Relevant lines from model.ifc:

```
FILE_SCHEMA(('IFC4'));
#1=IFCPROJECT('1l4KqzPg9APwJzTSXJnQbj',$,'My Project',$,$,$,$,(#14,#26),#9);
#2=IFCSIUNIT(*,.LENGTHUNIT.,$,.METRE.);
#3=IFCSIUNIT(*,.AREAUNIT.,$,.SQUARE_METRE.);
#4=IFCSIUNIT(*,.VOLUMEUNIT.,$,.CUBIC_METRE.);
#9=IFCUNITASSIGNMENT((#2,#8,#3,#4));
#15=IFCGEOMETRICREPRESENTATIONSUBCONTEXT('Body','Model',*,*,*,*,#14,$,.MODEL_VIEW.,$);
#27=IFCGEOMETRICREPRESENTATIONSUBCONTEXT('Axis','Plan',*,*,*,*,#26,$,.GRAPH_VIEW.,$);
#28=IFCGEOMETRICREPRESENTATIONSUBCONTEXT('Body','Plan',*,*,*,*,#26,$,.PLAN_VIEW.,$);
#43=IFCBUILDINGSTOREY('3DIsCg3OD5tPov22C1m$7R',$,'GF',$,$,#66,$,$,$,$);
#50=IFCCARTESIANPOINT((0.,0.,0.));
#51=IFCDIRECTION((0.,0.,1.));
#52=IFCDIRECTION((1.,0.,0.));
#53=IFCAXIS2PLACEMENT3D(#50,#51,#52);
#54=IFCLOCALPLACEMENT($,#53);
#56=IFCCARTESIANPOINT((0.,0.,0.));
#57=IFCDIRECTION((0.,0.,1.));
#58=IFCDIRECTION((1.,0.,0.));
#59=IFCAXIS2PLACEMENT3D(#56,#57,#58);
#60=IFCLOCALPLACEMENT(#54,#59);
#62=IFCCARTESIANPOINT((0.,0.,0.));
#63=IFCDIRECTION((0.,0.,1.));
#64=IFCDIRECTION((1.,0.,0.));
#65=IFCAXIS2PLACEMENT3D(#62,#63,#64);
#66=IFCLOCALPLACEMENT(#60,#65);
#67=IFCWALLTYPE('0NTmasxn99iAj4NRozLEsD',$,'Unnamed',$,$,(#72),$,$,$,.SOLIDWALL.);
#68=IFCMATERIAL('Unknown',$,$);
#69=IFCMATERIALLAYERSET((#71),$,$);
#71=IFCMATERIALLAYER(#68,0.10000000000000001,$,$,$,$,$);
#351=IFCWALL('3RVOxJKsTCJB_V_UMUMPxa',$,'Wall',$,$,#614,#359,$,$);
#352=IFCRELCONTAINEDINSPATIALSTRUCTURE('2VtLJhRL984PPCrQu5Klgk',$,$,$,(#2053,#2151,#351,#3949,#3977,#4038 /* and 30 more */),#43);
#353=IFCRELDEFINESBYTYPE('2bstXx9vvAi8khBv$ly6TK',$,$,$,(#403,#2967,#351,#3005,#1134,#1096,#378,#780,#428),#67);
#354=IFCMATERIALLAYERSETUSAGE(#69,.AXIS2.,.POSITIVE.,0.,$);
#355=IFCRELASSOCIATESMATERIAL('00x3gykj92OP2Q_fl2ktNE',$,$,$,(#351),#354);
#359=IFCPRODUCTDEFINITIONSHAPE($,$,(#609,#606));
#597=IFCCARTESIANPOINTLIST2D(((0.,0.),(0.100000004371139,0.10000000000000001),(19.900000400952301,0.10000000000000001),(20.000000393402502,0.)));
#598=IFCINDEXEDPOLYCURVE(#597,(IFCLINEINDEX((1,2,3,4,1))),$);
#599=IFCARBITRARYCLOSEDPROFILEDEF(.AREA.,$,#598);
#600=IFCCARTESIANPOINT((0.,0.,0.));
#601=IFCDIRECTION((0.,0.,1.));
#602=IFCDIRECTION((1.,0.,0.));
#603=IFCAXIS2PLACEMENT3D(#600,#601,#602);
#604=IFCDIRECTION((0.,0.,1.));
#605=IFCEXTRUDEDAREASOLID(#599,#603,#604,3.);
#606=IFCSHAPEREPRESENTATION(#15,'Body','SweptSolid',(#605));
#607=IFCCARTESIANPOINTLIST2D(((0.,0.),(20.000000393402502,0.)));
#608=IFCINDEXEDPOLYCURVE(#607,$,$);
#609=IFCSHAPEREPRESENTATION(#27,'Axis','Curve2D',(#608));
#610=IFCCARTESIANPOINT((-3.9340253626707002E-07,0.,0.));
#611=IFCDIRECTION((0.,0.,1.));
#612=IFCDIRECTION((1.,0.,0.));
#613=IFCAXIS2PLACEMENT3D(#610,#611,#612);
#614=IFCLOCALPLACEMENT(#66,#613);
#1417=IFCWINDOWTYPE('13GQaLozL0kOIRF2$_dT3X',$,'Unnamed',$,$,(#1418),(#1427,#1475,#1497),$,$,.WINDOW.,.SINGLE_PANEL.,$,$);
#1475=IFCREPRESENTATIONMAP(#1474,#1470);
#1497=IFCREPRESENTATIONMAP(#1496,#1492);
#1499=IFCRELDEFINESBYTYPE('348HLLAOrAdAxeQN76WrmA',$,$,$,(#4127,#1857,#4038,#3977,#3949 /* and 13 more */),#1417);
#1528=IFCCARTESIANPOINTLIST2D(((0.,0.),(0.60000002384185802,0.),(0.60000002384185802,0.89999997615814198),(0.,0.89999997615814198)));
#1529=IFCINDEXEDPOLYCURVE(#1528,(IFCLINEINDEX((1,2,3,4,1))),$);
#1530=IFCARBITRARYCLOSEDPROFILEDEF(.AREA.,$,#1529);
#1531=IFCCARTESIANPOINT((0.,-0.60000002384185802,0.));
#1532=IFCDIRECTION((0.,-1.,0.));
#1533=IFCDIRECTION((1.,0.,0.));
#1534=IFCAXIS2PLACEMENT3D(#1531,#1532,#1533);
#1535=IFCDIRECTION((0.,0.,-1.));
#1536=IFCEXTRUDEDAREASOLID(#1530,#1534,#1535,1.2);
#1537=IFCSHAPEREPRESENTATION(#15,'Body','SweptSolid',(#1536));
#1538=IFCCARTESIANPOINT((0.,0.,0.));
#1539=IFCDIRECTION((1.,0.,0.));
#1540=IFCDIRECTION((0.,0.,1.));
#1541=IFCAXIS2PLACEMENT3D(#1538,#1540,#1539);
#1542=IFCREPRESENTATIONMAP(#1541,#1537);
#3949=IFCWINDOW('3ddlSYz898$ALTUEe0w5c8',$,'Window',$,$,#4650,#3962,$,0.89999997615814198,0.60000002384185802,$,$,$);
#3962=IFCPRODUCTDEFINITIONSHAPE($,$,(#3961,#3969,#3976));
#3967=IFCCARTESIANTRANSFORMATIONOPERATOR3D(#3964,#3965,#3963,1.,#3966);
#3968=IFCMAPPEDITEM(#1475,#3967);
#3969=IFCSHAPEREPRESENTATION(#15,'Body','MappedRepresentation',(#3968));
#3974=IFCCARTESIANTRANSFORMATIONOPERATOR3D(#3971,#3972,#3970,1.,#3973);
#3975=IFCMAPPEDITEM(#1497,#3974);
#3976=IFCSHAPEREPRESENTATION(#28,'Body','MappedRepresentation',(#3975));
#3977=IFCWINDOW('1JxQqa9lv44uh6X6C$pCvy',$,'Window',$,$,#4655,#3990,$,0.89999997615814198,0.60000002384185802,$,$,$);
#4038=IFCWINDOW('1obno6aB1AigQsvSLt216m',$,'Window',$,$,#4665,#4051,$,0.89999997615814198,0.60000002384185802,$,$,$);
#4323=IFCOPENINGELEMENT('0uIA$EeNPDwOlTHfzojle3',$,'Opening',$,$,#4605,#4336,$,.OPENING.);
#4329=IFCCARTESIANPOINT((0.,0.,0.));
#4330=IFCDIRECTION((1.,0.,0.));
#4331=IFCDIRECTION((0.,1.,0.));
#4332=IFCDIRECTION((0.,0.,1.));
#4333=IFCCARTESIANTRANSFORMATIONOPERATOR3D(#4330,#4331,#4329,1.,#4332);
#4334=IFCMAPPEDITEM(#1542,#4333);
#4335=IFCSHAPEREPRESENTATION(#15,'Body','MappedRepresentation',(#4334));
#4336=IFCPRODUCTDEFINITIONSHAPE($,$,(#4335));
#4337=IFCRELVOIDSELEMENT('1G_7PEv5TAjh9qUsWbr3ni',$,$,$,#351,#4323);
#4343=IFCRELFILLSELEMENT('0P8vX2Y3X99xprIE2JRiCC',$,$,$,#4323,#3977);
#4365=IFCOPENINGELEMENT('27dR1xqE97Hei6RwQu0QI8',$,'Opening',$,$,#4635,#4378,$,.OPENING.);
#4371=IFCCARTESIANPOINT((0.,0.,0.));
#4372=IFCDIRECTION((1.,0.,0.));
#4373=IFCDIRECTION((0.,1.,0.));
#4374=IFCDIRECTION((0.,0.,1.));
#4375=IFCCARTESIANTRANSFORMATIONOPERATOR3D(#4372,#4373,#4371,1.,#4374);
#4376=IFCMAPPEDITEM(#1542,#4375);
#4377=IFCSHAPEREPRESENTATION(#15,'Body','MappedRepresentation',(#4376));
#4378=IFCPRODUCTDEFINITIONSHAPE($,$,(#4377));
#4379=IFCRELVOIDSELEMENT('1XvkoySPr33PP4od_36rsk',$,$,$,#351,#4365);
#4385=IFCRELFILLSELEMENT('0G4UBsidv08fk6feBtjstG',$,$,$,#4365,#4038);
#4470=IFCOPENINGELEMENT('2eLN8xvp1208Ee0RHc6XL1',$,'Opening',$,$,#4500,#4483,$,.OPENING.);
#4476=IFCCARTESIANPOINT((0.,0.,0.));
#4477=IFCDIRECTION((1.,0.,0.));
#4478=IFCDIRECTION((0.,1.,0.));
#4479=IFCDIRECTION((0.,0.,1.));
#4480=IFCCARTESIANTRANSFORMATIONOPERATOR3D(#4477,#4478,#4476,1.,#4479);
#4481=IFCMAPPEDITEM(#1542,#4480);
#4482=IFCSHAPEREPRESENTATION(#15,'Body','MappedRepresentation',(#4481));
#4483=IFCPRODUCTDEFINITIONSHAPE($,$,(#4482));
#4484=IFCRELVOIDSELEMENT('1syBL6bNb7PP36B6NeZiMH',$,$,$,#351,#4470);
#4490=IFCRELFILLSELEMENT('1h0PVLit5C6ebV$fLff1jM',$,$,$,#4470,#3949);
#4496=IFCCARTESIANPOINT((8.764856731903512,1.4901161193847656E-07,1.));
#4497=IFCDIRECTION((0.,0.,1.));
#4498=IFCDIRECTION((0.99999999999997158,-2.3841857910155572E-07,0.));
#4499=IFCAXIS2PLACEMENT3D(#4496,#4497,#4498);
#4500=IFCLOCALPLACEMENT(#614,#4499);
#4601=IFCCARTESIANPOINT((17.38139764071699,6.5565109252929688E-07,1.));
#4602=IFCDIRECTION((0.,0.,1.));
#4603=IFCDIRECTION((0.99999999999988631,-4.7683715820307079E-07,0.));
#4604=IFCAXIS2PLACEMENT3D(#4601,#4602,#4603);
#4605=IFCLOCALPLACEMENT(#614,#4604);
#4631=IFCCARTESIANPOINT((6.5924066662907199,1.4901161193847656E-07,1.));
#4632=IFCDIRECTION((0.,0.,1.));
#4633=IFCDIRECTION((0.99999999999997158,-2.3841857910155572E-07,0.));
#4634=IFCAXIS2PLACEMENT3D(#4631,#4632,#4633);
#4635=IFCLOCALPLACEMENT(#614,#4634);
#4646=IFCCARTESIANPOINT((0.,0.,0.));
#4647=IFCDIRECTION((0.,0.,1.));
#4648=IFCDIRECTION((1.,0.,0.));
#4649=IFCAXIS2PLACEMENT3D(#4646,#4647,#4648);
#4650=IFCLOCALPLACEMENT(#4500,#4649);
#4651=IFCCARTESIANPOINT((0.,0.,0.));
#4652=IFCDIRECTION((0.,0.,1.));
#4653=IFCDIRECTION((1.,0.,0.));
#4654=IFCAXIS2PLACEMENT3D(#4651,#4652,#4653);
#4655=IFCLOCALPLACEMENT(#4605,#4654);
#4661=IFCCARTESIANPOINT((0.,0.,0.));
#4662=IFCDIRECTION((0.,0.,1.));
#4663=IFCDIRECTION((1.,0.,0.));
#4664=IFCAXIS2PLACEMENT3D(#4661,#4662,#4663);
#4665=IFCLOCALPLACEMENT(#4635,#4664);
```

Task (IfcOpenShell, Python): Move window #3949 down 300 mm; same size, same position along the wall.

```python
import numpy as np
import ifcopenshell
import ifcopenshell.api.geometry
import ifcopenshell.util.placement
import ifcopenshell.util.unit

model = ifcopenshell.open("model.ifc")
unit_scale = ifcopenshell.util.unit.calculate_unit_scale(model)

window = model.by_guid("3ddlSYz898$ALTUEe0w5c8")
opening = window.FillsVoids[0].RelatingOpeningElement
dz = -0.3 / unit_scale

shift = np.array([0.0, 0.0, dz])
# The window is placed relative to its opening, so it follows when the opening moves.
matrix = ifcopenshell.util.placement.get_local_placement(opening.ObjectPlacement)
matrix[:3, 3] += shift
ifcopenshell.api.geometry.edit_object_placement(
    model, product=opening, matrix=matrix, is_si=False, should_transform_children=True
)

print(f"moved by {dz * unit_scale:+.3f} m")

model.write("model_rev.ifc")
```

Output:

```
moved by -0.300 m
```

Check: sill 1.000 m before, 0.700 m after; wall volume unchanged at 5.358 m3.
